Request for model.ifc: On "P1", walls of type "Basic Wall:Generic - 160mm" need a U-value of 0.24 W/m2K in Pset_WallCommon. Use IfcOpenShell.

First a look at what the model holds.

```python
import ifcopenshell
import ifcopenshell.util.element

model = ifcopenshell.open("model.ifc")
print(model.schema)
storey = next(s for s in model.by_type("IfcBuildingStorey") if s.Name == "P1")
walls = [e for e in ifcopenshell.util.element.get_decomposition(storey) if e.is_a("IfcWall")]
seen = {}
for e in walls:
    element_type = ifcopenshell.util.element.get_type(e)
    key = (element_type.Name if element_type != e and element_type else None, ifcopenshell.util.element.get_pset(e, "Pset_WallCommon", "ThermalTransmittance"))
    seen[key] = seen.get(key, 0) + 1
for (name, value), count in sorted(seen.items(), key=str):
    print(count, "x", name, "|", value)
```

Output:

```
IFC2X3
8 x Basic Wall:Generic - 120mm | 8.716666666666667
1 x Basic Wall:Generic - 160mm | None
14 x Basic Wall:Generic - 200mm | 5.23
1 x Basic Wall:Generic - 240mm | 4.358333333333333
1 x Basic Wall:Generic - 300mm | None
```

```python
import ifcopenshell
import ifcopenshell.api.pset
import ifcopenshell.util.element

model = ifcopenshell.open("model.ifc")

storey = next(s for s in model.by_type("IfcBuildingStorey") if s.Name == "P1")
walls = [e for e in ifcopenshell.util.element.get_decomposition(storey) if e.is_a("IfcWall")]

count = 0
for e in walls:
    element_type = ifcopenshell.util.element.get_type(e)
    if element_type in (None, e) or element_type.Name != "Basic Wall:Generic - 160mm":
        continue
    # add_pset returns the element's existing set when there is one.
    pset = ifcopenshell.api.pset.add_pset(model, product=e, name="Pset_WallCommon")
    ifcopenshell.api.pset.edit_pset(model, pset=pset, properties={"ThermalTransmittance": 0.24})
    count += 1

print(count, "walls updated")

model.write("model-out.ifc")
```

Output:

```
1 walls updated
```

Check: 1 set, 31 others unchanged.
